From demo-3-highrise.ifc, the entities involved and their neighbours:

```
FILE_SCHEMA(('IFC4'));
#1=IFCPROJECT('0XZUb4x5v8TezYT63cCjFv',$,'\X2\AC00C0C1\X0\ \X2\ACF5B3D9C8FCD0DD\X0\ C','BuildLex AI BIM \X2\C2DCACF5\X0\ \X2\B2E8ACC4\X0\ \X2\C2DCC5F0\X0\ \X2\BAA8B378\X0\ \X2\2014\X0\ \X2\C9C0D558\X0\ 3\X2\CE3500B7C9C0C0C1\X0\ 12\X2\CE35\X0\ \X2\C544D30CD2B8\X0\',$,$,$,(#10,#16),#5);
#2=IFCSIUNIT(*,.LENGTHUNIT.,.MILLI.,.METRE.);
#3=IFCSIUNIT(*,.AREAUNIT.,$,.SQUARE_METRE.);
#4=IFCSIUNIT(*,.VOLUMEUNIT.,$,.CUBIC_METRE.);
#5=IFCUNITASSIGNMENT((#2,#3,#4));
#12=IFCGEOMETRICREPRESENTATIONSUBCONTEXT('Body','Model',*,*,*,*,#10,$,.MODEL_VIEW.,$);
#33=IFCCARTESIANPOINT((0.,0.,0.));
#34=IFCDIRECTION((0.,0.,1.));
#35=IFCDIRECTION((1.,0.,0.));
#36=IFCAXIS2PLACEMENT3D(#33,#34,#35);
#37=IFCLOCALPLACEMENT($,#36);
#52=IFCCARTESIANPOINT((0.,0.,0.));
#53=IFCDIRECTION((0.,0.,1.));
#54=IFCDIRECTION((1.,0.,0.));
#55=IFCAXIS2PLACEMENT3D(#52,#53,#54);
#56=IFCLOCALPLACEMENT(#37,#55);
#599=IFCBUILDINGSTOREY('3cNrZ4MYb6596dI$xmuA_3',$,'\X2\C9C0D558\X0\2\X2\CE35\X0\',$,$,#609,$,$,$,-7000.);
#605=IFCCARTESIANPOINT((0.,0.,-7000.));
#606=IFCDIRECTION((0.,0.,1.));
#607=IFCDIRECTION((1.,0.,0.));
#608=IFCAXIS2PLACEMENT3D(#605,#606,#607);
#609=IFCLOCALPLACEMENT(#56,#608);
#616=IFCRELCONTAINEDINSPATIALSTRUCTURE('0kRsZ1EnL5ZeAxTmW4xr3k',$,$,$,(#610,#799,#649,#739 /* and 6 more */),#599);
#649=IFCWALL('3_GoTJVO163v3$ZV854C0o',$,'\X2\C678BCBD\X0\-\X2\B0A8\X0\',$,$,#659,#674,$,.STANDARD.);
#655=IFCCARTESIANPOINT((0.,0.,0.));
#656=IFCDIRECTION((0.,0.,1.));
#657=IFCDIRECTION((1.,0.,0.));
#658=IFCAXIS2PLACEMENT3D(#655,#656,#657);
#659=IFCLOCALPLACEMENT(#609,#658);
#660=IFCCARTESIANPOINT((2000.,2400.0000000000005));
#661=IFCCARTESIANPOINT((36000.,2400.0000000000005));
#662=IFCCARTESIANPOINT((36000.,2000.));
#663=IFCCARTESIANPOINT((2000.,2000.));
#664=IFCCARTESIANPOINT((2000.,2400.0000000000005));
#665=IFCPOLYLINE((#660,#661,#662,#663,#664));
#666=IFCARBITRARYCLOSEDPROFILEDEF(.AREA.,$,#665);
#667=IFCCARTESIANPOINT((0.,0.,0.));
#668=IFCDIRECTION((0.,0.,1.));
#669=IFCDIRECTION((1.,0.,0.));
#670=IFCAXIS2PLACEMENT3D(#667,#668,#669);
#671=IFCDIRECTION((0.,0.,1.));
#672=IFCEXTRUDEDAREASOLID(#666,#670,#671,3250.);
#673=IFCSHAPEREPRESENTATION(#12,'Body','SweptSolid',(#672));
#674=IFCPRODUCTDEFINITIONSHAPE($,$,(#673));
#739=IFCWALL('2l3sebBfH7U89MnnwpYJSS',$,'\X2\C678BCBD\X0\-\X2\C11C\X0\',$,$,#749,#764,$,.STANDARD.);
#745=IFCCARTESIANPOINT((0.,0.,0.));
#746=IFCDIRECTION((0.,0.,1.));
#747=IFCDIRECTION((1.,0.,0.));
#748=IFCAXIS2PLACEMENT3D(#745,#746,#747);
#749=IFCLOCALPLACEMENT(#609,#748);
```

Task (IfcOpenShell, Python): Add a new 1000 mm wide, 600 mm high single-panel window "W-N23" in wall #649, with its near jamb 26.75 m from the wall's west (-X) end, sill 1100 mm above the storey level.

```python
import numpy as np
import ifcopenshell
import ifcopenshell.api.feature
import ifcopenshell.api.geometry
import ifcopenshell.api.root
import ifcopenshell.api.spatial
import ifcopenshell.geom
import ifcopenshell.util.element
import ifcopenshell.util.placement
import ifcopenshell.util.representation
import ifcopenshell.util.shape
import ifcopenshell.util.unit

model = ifcopenshell.open("demo-3-highrise.ifc")
unit_scale = ifcopenshell.util.unit.calculate_unit_scale(model)
settings = ifcopenshell.geom.settings()


def volume(element):
    """Net volume in cubic metres, openings subtracted."""
    shape = ifcopenshell.geom.create_shape(settings, element)
    return ifcopenshell.util.shape.get_volume(shape.geometry)


wall = model.by_id(649)
storey = ifcopenshell.util.element.get_container(wall, ifc_class="IfcBuildingStorey")
context = ifcopenshell.util.representation.get_context(model, "Model", "Body", "MODEL_VIEW")
before = volume(wall)

width, height, from_end, sill = 1, 0.6, 26.75, 1.1  # metres

# The wall runs along its own X axis, and the end named is its -X end.
wall_shape = ifcopenshell.geom.create_shape(settings, wall)
x, y, z = ifcopenshell.util.shape.get_vertices(wall_shape.geometry).T
start = x.min() + from_end
face, thickness = float(y.min()), float(y.max() - y.min())
wall_matrix = ifcopenshell.util.placement.get_local_placement(wall.ObjectPlacement)
level = ifcopenshell.util.placement.get_local_placement(storey.ObjectPlacement)[2, 3]


def in_wall(x, y):
    """Placement at x, y metres in the wall's axes, at sill height."""
    matrix = wall_matrix.copy()
    matrix[:, 3] = wall_matrix @ np.array([x / unit_scale, y / unit_scale, 0.0, 1.0])
    matrix[2, 3] = level + sill / unit_scale
    return matrix


# Opening: a box that overshoots both wall faces by 50 mm.
opening = ifcopenshell.api.root.create_entity(model, ifc_class="IfcOpeningElement", predefined_type="OPENING")
box = ifcopenshell.api.geometry.add_wall_representation(
    model, context=context, length=width, height=height, thickness=thickness + 0.1
)
ifcopenshell.api.geometry.assign_representation(model, product=opening, representation=box)
ifcopenshell.api.geometry.edit_object_placement(model, product=opening, matrix=in_wall(start, face - 0.05), is_si=False)
ifcopenshell.api.feature.add_feature(model, feature=opening, element=wall)

window = ifcopenshell.api.root.create_entity(model, ifc_class="IfcWindow", name="W-N23", predefined_type="WINDOW")
window.OverallWidth, window.OverallHeight = width / unit_scale, height / unit_scale
window.PartitioningType = "SINGLE_PANEL"
body = ifcopenshell.api.geometry.add_window_representation(
    model,
    context=context,
    overall_width=window.OverallWidth,
    overall_height=window.OverallHeight,
    partition_type="SINGLE_PANEL",
)
ifcopenshell.api.geometry.assign_representation(model, product=window, representation=body)
ifcopenshell.api.spatial.assign_container(model, products=[window], relating_structure=storey)
ifcopenshell.api.feature.add_filling(model, opening=opening, element=window)

# Centre the window in the wall's thickness.
ifcopenshell.api.geometry.edit_object_placement(model, product=window, matrix=in_wall(start, face), is_si=False)
window_shape = ifcopenshell.geom.create_shape(settings, window)
depth = ifcopenshell.util.shape.get_vertices(window_shape.geometry)[:, 1]
offset = face + thickness / 2 - (depth.min() + depth.max()) / 2
ifcopenshell.api.geometry.edit_object_placement(model, product=window, matrix=in_wall(start, offset), is_si=False)

after = volume(wall)

print(f"wall volume {before:.3f} -> {after:.3f} m3")

model.write("demo-3-highrise_updated.ifc")
```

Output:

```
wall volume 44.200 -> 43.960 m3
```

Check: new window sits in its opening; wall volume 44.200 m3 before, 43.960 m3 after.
